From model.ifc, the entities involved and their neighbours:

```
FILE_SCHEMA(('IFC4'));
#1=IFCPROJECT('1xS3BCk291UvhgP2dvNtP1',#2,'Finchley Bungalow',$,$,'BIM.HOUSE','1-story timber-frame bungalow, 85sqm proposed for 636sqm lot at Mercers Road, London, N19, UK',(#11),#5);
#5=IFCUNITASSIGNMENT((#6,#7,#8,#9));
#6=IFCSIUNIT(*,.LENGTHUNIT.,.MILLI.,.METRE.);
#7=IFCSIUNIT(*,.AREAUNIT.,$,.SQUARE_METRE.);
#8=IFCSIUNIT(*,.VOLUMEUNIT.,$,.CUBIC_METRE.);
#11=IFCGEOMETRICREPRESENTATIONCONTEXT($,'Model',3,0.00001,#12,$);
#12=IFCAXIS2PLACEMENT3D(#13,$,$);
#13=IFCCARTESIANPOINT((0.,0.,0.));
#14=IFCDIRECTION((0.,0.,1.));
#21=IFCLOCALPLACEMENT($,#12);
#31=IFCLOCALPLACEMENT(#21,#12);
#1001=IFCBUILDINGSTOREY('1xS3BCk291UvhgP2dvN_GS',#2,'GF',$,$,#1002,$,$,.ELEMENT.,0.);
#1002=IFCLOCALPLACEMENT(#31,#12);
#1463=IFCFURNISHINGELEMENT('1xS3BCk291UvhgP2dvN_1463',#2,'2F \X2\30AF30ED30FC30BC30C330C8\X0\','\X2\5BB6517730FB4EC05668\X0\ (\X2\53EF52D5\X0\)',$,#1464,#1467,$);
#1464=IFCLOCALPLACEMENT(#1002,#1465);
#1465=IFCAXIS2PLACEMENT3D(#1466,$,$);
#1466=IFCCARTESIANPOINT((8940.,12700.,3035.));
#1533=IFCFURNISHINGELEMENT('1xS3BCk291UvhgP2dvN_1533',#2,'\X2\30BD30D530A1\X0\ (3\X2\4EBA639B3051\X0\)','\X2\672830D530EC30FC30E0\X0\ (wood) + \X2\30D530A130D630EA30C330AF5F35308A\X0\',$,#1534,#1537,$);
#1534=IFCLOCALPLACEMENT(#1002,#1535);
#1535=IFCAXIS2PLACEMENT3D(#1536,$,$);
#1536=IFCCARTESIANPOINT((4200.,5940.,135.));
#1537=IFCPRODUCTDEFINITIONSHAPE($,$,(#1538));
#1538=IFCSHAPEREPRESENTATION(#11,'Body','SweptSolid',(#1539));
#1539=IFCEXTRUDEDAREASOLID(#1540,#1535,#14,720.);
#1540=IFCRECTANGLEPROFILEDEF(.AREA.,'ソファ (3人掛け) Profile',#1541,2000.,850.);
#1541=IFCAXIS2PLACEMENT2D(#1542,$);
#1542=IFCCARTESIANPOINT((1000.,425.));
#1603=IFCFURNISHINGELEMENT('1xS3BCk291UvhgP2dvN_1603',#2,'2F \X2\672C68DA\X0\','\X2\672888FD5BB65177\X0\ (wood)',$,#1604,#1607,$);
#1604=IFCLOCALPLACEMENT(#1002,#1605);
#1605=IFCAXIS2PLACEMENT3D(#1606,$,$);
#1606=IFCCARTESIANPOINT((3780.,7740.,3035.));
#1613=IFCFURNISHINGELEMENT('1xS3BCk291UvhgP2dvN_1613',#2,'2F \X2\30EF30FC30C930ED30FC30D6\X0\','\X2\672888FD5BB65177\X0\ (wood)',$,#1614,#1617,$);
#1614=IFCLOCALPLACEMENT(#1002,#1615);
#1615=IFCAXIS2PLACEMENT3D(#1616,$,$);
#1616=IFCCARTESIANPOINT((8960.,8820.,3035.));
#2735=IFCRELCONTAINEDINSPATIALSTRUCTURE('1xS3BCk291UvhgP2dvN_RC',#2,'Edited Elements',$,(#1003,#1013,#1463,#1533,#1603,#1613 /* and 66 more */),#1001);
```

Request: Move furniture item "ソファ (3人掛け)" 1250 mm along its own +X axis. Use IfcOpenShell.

```python
import ifcopenshell
import ifcopenshell.api.geometry
import ifcopenshell.util.placement

model = ifcopenshell.open("model.ifc")

item = model.by_guid("1xS3BCk291UvhgP2dvN_1533")
matrix = ifcopenshell.util.placement.get_local_placement(item.ObjectPlacement)
matrix[:3, 3] += matrix[:3, 0] * 1250.0
ifcopenshell.api.geometry.edit_object_placement(model, product=item, matrix=matrix, is_si=False)

print(ifcopenshell.util.placement.get_local_placement(item.ObjectPlacement).round(3) + 0.0)

model.write("model-out.ifc")
```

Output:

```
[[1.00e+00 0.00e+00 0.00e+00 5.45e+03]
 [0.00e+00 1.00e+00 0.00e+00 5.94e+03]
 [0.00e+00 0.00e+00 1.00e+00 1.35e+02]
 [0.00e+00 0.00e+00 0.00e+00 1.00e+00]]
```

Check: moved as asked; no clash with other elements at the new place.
